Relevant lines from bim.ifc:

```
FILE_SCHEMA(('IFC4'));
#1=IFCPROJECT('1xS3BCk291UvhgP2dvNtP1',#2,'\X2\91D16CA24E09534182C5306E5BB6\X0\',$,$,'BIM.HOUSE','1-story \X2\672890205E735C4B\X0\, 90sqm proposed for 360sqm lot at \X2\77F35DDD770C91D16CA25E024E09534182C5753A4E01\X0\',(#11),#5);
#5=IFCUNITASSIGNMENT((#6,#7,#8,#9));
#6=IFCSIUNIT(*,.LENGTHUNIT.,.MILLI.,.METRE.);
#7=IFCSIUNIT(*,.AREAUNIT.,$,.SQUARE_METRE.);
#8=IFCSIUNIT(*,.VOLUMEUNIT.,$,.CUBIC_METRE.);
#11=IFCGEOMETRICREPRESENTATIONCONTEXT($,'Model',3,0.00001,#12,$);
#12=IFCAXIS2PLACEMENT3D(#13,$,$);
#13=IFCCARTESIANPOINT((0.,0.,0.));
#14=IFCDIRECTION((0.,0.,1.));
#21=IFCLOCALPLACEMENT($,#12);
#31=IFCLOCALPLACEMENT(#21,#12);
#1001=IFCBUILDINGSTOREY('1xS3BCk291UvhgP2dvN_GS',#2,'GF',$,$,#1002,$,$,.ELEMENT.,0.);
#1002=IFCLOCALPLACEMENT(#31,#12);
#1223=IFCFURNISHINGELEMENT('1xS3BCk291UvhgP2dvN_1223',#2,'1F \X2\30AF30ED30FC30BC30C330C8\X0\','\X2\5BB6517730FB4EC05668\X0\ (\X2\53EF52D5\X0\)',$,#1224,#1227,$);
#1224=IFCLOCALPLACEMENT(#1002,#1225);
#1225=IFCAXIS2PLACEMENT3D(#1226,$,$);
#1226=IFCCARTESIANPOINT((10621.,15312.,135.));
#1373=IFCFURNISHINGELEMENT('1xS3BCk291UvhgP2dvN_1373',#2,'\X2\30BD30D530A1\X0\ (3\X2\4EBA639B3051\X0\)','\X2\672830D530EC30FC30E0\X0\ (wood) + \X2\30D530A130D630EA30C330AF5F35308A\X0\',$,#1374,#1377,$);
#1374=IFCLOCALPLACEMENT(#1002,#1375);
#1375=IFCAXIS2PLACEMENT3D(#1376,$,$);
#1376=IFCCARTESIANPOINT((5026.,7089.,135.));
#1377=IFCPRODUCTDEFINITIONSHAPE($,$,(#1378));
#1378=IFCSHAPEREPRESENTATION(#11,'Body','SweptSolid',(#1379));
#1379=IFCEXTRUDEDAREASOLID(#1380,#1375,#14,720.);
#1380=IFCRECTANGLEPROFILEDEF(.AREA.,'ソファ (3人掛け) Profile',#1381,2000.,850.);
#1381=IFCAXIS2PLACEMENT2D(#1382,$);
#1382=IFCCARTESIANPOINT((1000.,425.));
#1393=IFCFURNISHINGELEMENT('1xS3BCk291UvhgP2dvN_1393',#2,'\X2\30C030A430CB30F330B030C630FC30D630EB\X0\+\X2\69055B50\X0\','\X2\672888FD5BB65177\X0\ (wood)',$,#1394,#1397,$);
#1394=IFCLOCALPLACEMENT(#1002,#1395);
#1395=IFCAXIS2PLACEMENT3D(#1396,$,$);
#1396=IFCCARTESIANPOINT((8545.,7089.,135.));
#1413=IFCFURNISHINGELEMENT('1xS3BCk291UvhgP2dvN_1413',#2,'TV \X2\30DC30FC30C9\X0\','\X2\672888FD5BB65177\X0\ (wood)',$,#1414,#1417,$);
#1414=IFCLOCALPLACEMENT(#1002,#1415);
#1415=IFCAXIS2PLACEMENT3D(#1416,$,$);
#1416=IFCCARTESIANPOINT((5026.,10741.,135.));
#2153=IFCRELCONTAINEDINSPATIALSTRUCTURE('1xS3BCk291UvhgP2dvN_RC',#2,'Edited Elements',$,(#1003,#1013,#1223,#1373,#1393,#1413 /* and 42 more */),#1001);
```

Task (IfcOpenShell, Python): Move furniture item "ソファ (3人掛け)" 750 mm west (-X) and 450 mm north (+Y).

```python
import ifcopenshell
import ifcopenshell.api.geometry
import ifcopenshell.util.placement
import ifcopenshell.util.unit

model = ifcopenshell.open("bim.ifc")
unit_scale = ifcopenshell.util.unit.calculate_unit_scale(model)

item = model.by_guid("1xS3BCk291UvhgP2dvN_1373")
matrix = ifcopenshell.util.placement.get_local_placement(item.ObjectPlacement)
matrix[0, 3] -= 0.75 / unit_scale
matrix[1, 3] += 0.45 / unit_scale
ifcopenshell.api.geometry.edit_object_placement(model, product=item, matrix=matrix, is_si=False)

print(ifcopenshell.util.placement.get_local_placement(item.ObjectPlacement).round(3) + 0.0)

model.write("bim_v2.ifc")
```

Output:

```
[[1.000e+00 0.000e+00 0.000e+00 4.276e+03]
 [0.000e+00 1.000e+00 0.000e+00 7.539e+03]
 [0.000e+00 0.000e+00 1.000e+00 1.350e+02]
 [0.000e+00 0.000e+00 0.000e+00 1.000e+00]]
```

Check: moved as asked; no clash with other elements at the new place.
